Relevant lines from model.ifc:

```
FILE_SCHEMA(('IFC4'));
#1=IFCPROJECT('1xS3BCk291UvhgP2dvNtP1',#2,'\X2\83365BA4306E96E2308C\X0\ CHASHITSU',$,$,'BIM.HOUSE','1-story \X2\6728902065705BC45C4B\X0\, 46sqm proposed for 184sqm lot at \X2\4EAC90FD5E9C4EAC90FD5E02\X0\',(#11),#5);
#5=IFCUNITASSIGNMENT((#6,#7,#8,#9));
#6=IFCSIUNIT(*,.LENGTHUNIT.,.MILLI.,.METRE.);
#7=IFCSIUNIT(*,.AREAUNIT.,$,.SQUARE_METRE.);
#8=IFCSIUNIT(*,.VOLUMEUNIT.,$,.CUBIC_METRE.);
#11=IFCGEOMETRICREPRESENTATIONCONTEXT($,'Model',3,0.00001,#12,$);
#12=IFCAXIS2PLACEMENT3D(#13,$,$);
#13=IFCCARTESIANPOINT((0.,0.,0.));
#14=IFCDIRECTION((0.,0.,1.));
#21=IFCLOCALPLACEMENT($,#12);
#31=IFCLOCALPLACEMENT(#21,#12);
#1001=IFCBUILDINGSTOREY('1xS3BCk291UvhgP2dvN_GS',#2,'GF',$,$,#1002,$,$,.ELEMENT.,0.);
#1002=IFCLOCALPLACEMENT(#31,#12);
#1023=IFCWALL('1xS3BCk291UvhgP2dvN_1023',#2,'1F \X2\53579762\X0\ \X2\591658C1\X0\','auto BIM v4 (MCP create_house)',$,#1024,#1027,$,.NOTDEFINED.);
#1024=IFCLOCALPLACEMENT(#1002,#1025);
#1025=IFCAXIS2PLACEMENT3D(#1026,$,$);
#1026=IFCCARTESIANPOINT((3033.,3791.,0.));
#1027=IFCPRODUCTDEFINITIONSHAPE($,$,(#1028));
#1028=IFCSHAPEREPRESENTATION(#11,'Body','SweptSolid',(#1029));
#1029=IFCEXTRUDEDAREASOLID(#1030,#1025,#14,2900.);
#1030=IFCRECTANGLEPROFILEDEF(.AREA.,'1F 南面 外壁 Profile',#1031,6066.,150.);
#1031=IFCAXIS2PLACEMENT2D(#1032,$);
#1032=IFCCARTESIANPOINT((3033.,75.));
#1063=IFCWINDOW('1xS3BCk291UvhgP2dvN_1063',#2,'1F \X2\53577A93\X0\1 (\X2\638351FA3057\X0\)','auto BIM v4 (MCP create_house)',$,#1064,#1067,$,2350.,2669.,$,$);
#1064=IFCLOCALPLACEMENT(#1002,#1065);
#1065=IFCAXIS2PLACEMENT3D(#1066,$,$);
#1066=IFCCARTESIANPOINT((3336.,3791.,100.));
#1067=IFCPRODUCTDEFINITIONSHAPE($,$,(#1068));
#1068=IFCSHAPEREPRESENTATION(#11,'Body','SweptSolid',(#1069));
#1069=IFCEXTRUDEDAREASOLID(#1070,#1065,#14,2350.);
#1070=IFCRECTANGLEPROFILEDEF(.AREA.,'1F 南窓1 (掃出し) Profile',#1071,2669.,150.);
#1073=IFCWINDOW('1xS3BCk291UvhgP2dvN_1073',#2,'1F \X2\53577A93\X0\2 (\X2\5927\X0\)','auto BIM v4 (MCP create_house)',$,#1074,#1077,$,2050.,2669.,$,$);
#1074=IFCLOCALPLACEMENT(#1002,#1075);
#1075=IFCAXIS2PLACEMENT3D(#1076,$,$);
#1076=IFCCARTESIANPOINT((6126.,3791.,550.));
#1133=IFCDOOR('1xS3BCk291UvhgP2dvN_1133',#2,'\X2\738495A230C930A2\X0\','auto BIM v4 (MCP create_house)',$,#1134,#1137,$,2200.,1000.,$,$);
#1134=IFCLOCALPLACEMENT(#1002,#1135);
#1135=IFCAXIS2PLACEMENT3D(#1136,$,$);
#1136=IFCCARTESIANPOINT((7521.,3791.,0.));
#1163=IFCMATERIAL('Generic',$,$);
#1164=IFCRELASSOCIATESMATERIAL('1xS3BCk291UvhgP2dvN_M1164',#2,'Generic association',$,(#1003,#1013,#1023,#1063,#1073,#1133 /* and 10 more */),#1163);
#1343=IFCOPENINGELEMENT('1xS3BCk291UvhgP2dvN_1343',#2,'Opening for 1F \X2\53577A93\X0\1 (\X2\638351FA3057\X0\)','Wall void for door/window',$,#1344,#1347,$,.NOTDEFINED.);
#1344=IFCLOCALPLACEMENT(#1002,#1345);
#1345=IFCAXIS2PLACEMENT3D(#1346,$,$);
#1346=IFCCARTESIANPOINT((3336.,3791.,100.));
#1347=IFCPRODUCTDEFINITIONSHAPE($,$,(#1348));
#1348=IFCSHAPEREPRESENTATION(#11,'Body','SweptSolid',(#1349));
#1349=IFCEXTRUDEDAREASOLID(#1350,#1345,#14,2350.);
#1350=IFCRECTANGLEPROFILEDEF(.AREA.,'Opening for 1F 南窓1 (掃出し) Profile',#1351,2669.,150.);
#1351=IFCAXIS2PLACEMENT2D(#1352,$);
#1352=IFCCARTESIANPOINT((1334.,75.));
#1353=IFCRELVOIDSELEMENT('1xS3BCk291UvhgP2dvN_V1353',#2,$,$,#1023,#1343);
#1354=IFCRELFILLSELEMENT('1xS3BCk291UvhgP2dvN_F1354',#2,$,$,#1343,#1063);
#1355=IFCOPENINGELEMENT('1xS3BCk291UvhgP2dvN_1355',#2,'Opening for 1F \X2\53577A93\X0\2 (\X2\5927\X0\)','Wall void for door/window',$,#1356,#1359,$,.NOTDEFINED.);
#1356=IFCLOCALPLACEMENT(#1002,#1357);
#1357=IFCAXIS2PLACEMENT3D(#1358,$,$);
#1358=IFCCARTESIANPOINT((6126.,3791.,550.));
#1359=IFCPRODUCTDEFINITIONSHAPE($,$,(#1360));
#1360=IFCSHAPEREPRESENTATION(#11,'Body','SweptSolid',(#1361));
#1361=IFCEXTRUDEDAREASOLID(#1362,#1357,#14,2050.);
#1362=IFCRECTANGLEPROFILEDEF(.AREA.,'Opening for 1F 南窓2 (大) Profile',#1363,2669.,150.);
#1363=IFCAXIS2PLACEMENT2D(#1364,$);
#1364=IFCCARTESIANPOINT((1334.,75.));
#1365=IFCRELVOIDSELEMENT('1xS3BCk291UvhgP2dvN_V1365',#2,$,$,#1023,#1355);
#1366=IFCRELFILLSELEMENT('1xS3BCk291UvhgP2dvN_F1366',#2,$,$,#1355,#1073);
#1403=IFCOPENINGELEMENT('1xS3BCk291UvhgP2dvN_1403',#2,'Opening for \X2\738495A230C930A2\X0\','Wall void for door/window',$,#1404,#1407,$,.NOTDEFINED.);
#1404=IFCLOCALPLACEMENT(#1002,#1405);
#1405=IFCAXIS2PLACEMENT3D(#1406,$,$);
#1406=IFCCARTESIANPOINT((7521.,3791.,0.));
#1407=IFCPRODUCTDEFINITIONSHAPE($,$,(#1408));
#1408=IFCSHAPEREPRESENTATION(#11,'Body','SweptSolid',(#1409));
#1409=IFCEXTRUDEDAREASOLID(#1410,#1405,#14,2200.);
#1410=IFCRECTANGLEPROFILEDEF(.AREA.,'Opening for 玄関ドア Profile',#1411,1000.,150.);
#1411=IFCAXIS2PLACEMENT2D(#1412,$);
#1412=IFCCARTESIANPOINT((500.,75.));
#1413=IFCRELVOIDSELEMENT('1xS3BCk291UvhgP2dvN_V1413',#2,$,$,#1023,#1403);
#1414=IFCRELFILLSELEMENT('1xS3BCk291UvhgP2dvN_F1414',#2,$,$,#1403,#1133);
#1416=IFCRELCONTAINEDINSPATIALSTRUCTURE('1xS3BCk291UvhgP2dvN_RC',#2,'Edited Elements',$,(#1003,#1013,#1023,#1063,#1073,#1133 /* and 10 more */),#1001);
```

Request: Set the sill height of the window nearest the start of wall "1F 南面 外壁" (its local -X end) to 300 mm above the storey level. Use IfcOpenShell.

```python
import numpy as np
import ifcopenshell
import ifcopenshell.api.geometry
import ifcopenshell.geom
import ifcopenshell.util.element
import ifcopenshell.util.placement
import ifcopenshell.util.shape
import ifcopenshell.util.unit

model = ifcopenshell.open("model.ifc")
unit_scale = ifcopenshell.util.unit.calculate_unit_scale(model)

window = model.by_guid("1xS3BCk291UvhgP2dvN_1063")
opening = window.FillsVoids[0].RelatingOpeningElement
storey = ifcopenshell.util.element.get_container(window, ifc_class="IfcBuildingStorey")
level = ifcopenshell.util.placement.get_local_placement(storey.ObjectPlacement)[2, 3]

# The opening's origin need not be at the sill, so measure its lowest point.
shape = ifcopenshell.geom.create_shape(ifcopenshell.geom.settings(), opening)
bottom = ifcopenshell.util.shape.get_shape_bottom_elevation(shape, shape.geometry) / unit_scale
dz = level + 300.0 - bottom

shift = np.array([0.0, 0.0, dz])
# The window is not placed relative to its opening, so move both.
for product in (opening, window):
    matrix = ifcopenshell.util.placement.get_local_placement(product.ObjectPlacement)
    matrix[:3, 3] += shift
    ifcopenshell.api.geometry.edit_object_placement(model, product=product, matrix=matrix, is_si=False)

print(f"moved by {dz * unit_scale:+.3f} m")

model.write("model_updated.ifc")
```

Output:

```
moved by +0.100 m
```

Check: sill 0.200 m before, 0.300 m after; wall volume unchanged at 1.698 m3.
